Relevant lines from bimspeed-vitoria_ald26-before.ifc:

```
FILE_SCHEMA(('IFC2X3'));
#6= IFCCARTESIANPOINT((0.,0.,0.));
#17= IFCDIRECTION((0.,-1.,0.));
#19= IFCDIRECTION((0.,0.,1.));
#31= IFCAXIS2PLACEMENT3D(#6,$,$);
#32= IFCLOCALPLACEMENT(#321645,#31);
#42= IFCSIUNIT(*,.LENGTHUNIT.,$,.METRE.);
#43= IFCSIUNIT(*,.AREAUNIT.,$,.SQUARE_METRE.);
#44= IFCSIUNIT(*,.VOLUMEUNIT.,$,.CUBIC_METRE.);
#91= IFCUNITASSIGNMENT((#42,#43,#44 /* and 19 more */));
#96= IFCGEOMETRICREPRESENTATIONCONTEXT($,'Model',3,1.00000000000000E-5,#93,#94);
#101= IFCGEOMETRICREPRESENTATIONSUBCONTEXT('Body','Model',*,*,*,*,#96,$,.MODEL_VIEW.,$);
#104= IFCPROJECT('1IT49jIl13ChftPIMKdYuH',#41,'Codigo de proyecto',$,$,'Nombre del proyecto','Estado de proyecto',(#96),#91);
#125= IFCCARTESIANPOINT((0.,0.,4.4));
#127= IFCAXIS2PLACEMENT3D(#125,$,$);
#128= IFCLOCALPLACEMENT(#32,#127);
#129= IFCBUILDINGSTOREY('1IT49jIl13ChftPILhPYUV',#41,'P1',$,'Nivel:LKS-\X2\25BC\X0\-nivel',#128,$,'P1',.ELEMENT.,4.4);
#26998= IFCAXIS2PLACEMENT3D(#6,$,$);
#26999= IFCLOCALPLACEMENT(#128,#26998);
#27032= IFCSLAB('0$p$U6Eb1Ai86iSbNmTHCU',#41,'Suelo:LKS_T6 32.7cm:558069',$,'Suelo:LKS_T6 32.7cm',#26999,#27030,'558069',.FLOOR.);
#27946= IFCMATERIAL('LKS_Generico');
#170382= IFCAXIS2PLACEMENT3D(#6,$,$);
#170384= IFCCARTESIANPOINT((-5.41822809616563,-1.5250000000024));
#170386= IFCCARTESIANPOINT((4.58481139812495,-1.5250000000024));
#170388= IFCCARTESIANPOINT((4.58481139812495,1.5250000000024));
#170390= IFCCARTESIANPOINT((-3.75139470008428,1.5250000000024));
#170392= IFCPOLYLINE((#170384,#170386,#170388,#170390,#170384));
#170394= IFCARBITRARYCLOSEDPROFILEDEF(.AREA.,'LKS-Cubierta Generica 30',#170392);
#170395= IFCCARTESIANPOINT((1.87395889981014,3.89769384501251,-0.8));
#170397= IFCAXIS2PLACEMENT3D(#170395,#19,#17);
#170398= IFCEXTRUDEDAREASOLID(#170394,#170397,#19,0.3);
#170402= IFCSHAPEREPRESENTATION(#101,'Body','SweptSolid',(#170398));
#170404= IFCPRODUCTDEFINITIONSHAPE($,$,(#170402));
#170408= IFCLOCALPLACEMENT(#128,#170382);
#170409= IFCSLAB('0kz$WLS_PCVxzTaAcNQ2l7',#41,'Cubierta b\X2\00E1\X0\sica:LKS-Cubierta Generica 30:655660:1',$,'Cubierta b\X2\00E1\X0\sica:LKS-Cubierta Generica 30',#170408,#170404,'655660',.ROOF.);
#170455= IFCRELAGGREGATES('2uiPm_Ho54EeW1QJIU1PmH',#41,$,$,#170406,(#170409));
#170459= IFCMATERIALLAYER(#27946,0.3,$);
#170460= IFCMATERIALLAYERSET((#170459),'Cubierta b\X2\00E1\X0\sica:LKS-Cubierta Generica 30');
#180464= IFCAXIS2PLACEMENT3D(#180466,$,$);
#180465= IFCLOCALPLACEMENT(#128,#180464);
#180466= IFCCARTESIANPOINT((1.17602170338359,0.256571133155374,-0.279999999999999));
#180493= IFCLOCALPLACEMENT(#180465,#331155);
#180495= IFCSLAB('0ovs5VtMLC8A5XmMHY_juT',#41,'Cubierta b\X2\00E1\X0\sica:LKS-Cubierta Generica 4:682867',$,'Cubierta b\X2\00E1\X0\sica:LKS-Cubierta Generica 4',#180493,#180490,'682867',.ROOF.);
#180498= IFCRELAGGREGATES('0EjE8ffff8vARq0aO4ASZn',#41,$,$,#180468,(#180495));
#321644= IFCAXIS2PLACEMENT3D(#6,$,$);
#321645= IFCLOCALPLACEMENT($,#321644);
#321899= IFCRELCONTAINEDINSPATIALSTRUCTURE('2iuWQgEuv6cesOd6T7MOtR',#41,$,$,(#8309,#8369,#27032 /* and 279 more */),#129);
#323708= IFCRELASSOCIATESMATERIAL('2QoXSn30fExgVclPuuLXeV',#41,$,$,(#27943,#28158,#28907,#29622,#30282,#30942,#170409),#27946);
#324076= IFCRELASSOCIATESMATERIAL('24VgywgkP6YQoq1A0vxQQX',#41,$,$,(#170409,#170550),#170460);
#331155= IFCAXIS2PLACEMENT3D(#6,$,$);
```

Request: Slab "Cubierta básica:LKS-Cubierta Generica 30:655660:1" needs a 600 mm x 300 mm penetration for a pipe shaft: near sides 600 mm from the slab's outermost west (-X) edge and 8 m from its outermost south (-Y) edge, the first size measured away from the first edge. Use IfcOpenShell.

```python
import numpy as np
import ifcopenshell
import ifcopenshell.api.feature
import ifcopenshell.api.geometry
import ifcopenshell.api.root
import ifcopenshell.geom
import ifcopenshell.util.placement
import ifcopenshell.util.representation
import ifcopenshell.util.shape
import ifcopenshell.util.unit

model = ifcopenshell.open("bimspeed-vitoria_ald26-before.ifc")
unit_scale = ifcopenshell.util.unit.calculate_unit_scale(model)
settings = ifcopenshell.geom.settings()


def volume(element):
    """Net volume in cubic metres, openings subtracted."""
    shape = ifcopenshell.geom.create_shape(settings, element)
    return ifcopenshell.util.shape.get_volume(shape.geometry)


slab = model.by_guid("0kz$WLS_PCVxzTaAcNQ2l7")
before = volume(slab)

# Extent in the slab's own axes, in metres. The edges named are its -X and -Y sides.
slab_shape = ifcopenshell.geom.create_shape(settings, slab)
vertices = ifcopenshell.util.shape.get_vertices(slab_shape.geometry)
x_min, y_min, bottom = vertices.min(axis=0)
top = vertices[:, 2].max()

opening = ifcopenshell.api.root.create_entity(model, ifc_class="IfcOpeningElement", name="Pipe shaft opening")
context = ifcopenshell.util.representation.get_context(model, "Model", "Body", "MODEL_VIEW")
width, depth = 0.6, 0.3
outline = [(0.0, 0.0), (width, 0.0), (width, depth), (0.0, depth), (0.0, 0.0)]
# Overshoot both faces by 50 mm so the cut is clean.
shape = ifcopenshell.api.geometry.add_slab_representation(
    model, context=context, depth=top - bottom + 0.1, polyline=outline
)
ifcopenshell.api.geometry.assign_representation(model, product=opening, representation=shape)

matrix = ifcopenshell.util.placement.get_local_placement(slab.ObjectPlacement)
matrix[:, 3] = matrix @ np.append(np.array([x_min + 0.6, y_min + 8, bottom - 0.05]) / unit_scale, 1.0)
ifcopenshell.api.geometry.edit_object_placement(model, product=opening, matrix=matrix, is_si=False)
ifcopenshell.api.feature.add_feature(model, feature=opening, element=slab)

after = volume(slab)

print(f"slab volume {before:.3f} -> {after:.3f} m3")

model.write("bimspeed-vitoria_ald26-before_v2.ifc")
```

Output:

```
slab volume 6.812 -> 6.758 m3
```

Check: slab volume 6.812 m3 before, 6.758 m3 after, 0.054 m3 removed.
